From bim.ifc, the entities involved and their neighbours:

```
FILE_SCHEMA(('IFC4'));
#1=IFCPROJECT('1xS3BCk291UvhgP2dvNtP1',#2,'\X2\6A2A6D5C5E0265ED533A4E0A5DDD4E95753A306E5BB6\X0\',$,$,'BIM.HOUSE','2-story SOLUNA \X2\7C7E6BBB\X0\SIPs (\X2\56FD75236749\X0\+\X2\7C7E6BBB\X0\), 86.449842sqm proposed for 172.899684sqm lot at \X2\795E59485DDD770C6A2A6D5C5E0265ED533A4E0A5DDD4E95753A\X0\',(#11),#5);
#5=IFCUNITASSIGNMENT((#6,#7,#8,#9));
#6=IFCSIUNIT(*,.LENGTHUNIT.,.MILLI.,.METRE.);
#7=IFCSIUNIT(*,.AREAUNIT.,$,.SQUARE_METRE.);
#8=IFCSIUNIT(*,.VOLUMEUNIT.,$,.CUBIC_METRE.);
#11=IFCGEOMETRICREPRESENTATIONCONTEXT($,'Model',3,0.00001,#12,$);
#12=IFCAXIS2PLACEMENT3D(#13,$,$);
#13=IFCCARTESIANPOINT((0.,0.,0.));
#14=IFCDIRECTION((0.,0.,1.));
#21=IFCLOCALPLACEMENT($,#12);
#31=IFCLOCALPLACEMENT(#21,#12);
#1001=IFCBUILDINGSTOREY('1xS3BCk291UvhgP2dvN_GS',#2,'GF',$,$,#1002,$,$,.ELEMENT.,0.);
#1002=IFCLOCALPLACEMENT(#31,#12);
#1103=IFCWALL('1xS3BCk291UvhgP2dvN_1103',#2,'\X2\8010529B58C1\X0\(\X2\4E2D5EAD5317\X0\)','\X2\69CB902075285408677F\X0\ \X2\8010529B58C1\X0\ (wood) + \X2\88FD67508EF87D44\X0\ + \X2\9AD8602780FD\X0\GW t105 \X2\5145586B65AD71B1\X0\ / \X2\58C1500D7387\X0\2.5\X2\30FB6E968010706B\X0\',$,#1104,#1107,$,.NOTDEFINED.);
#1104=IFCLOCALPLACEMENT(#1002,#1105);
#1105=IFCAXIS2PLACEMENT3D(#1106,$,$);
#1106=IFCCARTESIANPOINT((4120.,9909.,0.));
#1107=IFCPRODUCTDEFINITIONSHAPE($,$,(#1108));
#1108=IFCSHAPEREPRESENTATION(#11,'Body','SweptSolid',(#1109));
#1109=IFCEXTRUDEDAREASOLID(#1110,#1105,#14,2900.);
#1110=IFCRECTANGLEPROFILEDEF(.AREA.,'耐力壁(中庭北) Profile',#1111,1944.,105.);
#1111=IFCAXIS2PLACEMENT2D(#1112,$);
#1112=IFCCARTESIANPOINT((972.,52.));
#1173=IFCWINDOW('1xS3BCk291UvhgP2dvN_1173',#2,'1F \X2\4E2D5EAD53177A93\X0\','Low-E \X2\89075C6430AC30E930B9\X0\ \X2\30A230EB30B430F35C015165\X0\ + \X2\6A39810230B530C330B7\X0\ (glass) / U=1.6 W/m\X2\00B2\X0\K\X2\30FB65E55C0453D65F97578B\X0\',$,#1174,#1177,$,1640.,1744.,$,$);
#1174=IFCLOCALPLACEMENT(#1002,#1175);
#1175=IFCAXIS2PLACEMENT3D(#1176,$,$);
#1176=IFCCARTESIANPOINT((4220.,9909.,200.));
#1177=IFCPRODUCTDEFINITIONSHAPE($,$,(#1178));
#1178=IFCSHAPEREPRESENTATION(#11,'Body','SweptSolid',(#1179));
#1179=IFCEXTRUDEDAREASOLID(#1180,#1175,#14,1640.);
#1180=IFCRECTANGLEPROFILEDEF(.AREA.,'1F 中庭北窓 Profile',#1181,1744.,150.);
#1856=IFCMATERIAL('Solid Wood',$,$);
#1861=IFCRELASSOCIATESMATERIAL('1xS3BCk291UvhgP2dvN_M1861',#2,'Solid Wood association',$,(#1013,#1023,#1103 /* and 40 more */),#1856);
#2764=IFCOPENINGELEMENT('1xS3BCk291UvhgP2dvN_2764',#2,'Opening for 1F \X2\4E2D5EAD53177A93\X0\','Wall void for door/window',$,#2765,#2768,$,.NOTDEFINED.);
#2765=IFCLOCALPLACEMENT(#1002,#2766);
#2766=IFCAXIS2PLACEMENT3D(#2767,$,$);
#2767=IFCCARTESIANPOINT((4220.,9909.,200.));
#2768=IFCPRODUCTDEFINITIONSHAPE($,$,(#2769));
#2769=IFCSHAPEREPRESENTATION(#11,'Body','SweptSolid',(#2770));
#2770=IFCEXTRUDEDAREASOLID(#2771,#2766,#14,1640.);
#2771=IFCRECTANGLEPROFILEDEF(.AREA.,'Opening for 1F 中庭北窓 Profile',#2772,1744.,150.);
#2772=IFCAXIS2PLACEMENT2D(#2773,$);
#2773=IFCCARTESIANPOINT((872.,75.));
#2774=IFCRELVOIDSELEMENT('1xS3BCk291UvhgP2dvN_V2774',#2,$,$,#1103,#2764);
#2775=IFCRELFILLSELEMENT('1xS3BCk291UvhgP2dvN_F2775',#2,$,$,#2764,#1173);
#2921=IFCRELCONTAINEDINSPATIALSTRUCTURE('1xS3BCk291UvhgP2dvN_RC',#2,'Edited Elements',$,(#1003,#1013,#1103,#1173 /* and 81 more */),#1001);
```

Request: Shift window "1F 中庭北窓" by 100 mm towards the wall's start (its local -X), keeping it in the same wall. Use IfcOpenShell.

```python
import ifcopenshell
import ifcopenshell.api.geometry
import ifcopenshell.util.placement
import ifcopenshell.util.unit

model = ifcopenshell.open("bim.ifc")
unit_scale = ifcopenshell.util.unit.calculate_unit_scale(model)

window = model.by_guid("1xS3BCk291UvhgP2dvN_1173")
opening = window.FillsVoids[0].RelatingOpeningElement
wall = opening.VoidsElements[0].RelatingBuildingElement

wall_matrix = ifcopenshell.util.placement.get_local_placement(wall.ObjectPlacement)
shift = wall_matrix[:3, 0] * -0.1 / unit_scale
before = ifcopenshell.util.placement.get_local_placement(window.ObjectPlacement)[:3, 3].copy()

# The window is not placed relative to its opening, so move both.
for product in (opening, window):
    matrix = ifcopenshell.util.placement.get_local_placement(product.ObjectPlacement)
    matrix[:3, 3] += shift
    ifcopenshell.api.geometry.edit_object_placement(model, product=product, matrix=matrix, is_si=False)

after = ifcopenshell.util.placement.get_local_placement(window.ObjectPlacement)[:3, 3]
print("window moved by", (after - before).round(3) + 0.0)

model.write("bim_rev.ifc")
```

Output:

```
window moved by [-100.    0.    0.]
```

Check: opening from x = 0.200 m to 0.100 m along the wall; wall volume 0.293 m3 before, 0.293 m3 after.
